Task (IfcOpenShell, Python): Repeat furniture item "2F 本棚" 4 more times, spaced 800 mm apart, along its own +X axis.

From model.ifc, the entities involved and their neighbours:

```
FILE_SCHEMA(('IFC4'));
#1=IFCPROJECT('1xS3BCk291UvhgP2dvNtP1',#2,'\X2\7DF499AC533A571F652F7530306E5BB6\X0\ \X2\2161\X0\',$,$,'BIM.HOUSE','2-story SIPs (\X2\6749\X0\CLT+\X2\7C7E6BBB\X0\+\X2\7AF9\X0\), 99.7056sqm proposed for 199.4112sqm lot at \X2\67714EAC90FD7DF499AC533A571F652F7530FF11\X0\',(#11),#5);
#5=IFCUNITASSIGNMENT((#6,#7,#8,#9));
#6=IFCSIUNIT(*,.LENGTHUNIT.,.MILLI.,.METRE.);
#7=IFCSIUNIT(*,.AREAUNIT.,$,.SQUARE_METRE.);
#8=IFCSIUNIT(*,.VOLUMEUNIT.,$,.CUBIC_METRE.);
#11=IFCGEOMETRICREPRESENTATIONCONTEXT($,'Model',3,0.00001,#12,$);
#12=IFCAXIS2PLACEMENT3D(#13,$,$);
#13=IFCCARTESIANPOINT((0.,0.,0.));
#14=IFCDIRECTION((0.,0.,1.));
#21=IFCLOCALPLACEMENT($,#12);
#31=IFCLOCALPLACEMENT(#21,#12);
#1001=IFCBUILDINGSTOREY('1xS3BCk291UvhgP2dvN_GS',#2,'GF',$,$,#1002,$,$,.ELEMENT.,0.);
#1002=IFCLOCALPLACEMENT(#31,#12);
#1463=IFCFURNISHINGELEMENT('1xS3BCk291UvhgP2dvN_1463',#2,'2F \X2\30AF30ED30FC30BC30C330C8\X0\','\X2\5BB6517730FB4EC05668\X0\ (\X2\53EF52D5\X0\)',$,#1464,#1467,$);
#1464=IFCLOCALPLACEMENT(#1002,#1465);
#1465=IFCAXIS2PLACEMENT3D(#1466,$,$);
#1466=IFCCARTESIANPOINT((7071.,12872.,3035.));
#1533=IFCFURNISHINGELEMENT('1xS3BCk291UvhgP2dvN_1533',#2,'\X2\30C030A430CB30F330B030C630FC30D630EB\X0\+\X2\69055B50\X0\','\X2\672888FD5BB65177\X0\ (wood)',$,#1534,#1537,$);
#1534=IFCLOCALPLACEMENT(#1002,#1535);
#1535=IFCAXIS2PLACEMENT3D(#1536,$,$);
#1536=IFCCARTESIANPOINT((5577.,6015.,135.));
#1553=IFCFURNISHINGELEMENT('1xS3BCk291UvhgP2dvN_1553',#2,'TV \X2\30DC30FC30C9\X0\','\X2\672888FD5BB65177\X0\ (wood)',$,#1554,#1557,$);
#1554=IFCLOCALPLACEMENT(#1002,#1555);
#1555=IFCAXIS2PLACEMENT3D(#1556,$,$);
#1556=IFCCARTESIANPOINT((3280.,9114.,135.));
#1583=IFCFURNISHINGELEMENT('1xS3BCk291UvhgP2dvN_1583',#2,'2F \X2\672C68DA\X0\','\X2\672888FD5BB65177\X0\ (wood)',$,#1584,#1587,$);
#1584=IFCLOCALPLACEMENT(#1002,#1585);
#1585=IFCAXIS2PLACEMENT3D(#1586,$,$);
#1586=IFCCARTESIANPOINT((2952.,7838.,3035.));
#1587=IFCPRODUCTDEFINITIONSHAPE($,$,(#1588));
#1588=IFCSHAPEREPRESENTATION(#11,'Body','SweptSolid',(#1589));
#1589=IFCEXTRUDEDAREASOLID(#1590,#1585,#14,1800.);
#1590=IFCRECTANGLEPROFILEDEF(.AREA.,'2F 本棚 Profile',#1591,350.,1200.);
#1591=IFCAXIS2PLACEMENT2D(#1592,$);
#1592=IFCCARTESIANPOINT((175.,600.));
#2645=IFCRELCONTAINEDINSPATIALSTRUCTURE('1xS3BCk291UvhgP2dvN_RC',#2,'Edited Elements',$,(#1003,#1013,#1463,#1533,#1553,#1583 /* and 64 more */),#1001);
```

```python
import ifcopenshell
import ifcopenshell.api.geometry
import ifcopenshell.api.root
import ifcopenshell.util.element
import ifcopenshell.util.placement
import ifcopenshell.util.unit

model = ifcopenshell.open("model.ifc")
unit_scale = ifcopenshell.util.unit.calculate_unit_scale(model)


def reuse_history(source, copy):
    """copy_class also copies each property set's owner history, people and application; keep the originals."""
    for rel in copy.IsDefinedBy:
        if rel.is_a("IfcRelDefinesByProperties") and (history := rel.RelatingPropertyDefinition.OwnerHistory):
            rel.RelatingPropertyDefinition.OwnerHistory = source.OwnerHistory
            ifcopenshell.util.element.remove_deep2(model, history)


source = model.by_guid("1xS3BCk291UvhgP2dvN_1583")
base = ifcopenshell.util.placement.get_local_placement(source.ObjectPlacement)
step = base[:3, 0] * 0.8 / unit_scale

for i in range(1, 5):
    copy = ifcopenshell.api.root.copy_class(model, product=source)
    copy.Representation = ifcopenshell.util.element.copy_deep(
        model, source.Representation, exclude=["IfcGeometricRepresentationContext", "IfcRepresentationMap"]
    )
    reuse_history(source, copy)
    matrix = base.copy()
    matrix[:3, 3] += i * step
    print("added at", matrix[:3, 3].round(3) + 0.0)
    ifcopenshell.api.geometry.edit_object_placement(model, product=copy, matrix=matrix, is_si=False)

model.write("model_edited.ifc")
```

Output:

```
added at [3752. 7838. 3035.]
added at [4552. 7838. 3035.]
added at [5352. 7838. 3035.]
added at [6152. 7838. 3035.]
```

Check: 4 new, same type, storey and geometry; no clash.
